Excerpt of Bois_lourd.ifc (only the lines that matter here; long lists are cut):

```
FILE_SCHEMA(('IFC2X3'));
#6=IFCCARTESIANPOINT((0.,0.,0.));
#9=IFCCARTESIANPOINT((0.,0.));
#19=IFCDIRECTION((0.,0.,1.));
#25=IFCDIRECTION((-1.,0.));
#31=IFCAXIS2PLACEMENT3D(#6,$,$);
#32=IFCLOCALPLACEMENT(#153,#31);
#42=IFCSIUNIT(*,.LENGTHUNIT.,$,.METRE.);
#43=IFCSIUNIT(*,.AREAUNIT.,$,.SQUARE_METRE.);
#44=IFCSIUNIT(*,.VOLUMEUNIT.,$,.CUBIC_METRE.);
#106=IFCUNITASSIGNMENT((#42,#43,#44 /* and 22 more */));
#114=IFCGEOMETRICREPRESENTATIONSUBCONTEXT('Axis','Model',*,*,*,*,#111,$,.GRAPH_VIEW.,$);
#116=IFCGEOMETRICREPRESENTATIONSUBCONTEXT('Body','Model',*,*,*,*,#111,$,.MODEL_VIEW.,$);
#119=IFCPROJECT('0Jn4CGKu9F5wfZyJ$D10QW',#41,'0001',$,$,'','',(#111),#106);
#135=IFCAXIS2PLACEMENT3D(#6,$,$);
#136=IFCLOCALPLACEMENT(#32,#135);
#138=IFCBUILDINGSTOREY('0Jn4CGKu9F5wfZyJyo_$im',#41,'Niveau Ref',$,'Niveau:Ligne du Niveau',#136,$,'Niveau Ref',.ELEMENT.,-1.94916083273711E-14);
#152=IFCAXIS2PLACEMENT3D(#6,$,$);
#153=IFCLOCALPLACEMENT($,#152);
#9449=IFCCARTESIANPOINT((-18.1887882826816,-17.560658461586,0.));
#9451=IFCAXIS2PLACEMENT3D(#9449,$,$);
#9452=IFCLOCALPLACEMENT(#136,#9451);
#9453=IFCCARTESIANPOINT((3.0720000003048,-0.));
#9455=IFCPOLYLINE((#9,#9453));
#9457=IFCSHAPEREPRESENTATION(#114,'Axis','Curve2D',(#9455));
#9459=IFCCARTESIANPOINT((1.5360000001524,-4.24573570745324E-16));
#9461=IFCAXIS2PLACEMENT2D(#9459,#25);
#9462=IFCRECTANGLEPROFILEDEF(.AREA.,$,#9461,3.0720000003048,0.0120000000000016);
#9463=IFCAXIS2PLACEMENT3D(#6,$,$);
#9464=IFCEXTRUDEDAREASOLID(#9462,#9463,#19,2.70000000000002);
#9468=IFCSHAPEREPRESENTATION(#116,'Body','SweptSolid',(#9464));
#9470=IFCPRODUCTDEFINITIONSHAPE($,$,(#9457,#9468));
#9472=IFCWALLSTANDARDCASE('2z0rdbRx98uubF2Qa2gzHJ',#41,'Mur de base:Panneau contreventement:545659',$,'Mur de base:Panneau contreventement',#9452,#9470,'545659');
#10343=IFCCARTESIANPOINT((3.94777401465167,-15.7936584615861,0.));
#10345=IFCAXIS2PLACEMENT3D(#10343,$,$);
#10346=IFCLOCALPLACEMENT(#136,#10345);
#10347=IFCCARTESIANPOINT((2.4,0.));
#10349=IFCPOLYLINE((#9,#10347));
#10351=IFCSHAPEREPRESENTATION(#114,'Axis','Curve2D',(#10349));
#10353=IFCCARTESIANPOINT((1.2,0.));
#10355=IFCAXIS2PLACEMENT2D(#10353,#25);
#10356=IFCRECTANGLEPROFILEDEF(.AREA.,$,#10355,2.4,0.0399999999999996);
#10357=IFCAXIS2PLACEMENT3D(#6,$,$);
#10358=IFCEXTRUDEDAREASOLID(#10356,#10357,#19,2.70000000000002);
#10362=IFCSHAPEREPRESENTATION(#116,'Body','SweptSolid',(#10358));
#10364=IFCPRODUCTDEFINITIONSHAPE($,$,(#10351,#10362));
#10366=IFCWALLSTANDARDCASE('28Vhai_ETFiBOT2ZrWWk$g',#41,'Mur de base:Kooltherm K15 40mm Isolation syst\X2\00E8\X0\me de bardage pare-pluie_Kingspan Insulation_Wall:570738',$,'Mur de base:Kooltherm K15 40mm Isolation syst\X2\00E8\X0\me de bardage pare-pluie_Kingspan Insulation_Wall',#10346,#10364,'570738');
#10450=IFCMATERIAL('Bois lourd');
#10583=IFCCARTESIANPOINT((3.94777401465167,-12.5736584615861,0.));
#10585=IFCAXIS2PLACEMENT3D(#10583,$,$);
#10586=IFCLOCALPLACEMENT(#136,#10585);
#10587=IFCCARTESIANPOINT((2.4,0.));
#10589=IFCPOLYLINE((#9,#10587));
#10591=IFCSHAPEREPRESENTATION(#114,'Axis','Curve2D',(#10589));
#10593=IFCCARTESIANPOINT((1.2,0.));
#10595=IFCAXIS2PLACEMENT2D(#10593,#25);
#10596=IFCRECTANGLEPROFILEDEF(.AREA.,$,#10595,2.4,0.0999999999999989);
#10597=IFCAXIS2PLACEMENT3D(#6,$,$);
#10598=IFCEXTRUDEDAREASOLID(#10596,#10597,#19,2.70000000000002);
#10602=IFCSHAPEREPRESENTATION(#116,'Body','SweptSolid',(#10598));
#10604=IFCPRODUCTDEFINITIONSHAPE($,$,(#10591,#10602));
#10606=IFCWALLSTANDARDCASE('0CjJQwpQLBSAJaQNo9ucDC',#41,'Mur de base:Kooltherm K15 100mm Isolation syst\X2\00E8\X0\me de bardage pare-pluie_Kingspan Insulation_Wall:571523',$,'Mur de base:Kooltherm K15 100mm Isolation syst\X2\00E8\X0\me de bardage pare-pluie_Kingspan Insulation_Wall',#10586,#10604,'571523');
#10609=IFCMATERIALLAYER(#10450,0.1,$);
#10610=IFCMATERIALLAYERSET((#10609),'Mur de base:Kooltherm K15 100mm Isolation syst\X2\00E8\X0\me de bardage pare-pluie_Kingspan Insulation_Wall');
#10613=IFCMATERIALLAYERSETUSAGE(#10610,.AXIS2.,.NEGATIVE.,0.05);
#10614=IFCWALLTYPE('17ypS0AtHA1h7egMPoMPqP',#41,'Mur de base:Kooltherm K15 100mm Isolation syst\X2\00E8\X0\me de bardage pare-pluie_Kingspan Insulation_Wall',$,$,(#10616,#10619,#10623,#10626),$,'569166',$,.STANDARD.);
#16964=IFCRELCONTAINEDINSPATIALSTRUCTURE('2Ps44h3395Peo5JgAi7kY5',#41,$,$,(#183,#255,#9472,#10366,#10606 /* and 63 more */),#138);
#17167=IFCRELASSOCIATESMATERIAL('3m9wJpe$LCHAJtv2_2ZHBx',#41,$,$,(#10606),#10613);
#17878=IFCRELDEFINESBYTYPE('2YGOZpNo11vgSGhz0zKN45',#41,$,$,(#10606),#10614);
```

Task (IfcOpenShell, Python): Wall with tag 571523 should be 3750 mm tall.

```python
import ifcopenshell
import ifcopenshell.geom
import ifcopenshell.util.representation
import ifcopenshell.util.shape
import ifcopenshell.util.unit

model = ifcopenshell.open("Bois_lourd.ifc")
unit_scale = ifcopenshell.util.unit.calculate_unit_scale(model)
settings = ifcopenshell.geom.settings()


def volume(element):
    """Net volume in cubic metres, openings subtracted."""
    shape = ifcopenshell.geom.create_shape(settings, element)
    return ifcopenshell.util.shape.get_volume(shape.geometry)


wall = model.by_guid("0CjJQwpQLBSAJaQNo9ucDC")
before = volume(wall)

body = ifcopenshell.util.representation.get_representation(wall, "Model", "Body")
solid = body.Items[0]
old_height = solid.Depth
solid.Depth = 3.75 / unit_scale
after = volume(wall)

print(f"height {old_height:g} -> {solid.Depth:g}, volume {before:.3f} -> {after:.3f} m3")

model.write("Bois_lourd_v2.ifc")
```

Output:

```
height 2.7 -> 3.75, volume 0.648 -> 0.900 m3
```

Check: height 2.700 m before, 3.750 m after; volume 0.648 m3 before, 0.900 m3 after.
